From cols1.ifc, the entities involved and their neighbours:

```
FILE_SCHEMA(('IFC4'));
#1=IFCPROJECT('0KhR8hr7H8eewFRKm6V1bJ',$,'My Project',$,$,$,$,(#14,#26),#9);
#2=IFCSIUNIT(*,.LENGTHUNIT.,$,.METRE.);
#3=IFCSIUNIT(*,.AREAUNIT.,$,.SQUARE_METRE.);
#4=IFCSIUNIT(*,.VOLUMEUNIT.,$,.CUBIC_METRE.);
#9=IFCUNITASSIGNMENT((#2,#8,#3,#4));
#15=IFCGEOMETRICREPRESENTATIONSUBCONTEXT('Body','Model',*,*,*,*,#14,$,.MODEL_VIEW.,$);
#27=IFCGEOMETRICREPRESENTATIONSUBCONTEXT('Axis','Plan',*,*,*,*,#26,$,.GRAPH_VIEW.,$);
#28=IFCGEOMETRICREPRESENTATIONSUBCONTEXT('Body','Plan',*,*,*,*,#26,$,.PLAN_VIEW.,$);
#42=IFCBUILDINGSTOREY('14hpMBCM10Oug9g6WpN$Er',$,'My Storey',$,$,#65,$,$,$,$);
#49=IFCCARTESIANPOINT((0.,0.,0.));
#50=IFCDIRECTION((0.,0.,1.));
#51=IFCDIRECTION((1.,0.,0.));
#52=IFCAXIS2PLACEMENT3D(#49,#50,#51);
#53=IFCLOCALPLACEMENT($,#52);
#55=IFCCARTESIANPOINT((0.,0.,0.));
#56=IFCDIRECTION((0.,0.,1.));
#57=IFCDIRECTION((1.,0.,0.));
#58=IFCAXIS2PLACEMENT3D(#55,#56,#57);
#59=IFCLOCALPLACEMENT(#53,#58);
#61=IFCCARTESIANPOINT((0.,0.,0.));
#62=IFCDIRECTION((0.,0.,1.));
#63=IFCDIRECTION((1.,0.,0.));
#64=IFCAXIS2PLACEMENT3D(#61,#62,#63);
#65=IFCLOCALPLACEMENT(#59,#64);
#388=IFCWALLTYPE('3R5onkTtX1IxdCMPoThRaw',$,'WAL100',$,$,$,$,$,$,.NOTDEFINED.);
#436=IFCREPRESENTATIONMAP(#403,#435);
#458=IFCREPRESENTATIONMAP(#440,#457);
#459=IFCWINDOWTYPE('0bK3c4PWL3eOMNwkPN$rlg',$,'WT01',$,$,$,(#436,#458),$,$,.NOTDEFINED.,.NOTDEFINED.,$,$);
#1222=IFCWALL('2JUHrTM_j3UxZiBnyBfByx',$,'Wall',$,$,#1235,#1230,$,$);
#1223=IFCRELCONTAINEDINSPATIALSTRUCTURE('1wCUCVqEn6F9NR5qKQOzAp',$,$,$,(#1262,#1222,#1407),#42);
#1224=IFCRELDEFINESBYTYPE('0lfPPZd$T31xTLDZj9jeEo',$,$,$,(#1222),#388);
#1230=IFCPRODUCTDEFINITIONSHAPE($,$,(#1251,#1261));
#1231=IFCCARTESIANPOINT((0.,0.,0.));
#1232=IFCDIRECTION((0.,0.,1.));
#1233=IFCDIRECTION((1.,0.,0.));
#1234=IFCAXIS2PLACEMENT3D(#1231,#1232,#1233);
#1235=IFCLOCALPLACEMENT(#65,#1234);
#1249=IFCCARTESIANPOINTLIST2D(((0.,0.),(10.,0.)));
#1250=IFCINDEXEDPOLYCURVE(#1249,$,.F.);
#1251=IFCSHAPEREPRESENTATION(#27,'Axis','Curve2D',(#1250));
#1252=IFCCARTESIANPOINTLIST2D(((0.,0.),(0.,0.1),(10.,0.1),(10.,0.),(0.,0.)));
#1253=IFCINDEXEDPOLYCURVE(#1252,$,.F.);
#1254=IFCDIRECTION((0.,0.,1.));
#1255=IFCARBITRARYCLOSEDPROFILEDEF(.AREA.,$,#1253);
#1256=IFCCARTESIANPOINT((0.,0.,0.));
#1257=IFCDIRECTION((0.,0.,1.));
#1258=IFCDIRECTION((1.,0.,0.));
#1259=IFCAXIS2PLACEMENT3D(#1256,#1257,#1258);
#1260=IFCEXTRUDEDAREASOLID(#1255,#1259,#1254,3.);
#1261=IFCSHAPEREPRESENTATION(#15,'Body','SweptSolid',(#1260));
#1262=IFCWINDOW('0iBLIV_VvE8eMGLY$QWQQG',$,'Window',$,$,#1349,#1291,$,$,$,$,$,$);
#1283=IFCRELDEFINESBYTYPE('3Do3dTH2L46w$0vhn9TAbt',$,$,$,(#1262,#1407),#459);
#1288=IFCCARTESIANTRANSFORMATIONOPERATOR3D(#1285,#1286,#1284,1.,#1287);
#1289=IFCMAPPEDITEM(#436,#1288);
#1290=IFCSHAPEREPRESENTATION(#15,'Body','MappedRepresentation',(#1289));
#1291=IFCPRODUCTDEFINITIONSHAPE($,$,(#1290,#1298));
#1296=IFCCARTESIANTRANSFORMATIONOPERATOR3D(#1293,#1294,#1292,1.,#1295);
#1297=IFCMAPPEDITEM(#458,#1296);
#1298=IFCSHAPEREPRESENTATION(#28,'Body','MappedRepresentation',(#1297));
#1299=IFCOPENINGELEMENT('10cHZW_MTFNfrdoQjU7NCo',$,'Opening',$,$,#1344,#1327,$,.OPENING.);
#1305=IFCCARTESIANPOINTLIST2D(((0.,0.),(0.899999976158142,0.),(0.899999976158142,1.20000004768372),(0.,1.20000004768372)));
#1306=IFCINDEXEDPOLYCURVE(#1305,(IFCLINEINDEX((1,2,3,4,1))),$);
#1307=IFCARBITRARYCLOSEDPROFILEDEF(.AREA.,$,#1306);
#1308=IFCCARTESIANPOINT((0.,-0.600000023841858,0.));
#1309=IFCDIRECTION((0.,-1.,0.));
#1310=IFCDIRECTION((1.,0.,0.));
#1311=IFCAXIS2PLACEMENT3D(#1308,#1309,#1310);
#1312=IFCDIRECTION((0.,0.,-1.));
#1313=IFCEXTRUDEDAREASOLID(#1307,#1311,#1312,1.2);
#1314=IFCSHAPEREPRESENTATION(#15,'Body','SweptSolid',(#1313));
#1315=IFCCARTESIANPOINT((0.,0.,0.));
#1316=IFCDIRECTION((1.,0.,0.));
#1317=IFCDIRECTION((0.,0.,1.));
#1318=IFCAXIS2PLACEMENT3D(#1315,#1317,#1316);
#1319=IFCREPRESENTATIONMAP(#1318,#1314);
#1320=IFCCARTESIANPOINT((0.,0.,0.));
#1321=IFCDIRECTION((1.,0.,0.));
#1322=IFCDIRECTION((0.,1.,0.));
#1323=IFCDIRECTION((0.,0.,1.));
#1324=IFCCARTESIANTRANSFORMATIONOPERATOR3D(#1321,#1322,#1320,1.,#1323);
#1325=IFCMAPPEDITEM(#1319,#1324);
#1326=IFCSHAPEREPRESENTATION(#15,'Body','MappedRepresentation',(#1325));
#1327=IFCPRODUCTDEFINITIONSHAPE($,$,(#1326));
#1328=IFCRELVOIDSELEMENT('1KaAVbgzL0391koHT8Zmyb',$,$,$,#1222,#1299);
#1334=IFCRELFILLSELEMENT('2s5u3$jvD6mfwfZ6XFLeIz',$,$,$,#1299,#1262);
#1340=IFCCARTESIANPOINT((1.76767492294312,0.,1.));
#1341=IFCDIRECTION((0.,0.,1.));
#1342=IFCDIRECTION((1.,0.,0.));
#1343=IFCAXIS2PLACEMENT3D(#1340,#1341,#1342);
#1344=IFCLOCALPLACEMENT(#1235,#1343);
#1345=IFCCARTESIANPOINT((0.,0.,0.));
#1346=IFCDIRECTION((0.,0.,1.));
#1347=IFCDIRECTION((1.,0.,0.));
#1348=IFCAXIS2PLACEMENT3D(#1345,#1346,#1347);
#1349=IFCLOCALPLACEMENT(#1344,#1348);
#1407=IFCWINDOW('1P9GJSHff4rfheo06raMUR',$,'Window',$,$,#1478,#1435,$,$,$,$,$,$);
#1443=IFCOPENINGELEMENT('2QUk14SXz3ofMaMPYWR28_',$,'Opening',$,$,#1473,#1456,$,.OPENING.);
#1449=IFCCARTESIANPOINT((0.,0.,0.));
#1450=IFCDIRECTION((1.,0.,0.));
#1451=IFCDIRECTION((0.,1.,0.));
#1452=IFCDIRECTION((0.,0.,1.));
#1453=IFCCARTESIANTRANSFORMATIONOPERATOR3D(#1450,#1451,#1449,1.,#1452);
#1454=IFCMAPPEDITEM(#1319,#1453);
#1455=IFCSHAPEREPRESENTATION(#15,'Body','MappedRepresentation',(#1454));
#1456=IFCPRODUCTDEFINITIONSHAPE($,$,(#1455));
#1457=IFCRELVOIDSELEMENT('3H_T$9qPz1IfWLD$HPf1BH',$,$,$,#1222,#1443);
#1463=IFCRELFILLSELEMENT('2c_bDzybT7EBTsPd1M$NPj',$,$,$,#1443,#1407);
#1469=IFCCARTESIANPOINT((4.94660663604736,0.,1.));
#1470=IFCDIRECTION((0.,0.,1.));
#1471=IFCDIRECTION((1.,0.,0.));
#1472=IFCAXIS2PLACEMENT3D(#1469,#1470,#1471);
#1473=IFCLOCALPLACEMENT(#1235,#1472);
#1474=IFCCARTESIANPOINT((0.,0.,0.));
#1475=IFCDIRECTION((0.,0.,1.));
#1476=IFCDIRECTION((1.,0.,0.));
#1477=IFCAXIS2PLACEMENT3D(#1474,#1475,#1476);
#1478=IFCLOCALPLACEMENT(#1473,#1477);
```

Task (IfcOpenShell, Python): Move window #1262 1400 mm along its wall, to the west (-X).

```python
import ifcopenshell
import ifcopenshell.api.geometry
import ifcopenshell.util.placement
import ifcopenshell.util.unit

model = ifcopenshell.open("cols1.ifc")
unit_scale = ifcopenshell.util.unit.calculate_unit_scale(model)

window = model.by_id(1262)
opening = window.FillsVoids[0].RelatingOpeningElement
wall = opening.VoidsElements[0].RelatingBuildingElement

wall_matrix = ifcopenshell.util.placement.get_local_placement(wall.ObjectPlacement)
shift = wall_matrix[:3, 0] * -1.4 / unit_scale
before = ifcopenshell.util.placement.get_local_placement(window.ObjectPlacement)[:3, 3].copy()

# The window is placed relative to its opening, so it follows when the opening moves.
matrix = ifcopenshell.util.placement.get_local_placement(opening.ObjectPlacement)
matrix[:3, 3] += shift
ifcopenshell.api.geometry.edit_object_placement(
    model, product=opening, matrix=matrix, is_si=False, should_transform_children=True
)

after = ifcopenshell.util.placement.get_local_placement(window.ObjectPlacement)[:3, 3]
print("window moved by", (after - before).round(3) + 0.0)

model.write("cols1_rev.ifc")
```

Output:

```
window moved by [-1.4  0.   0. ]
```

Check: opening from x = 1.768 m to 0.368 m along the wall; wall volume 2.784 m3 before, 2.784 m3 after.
